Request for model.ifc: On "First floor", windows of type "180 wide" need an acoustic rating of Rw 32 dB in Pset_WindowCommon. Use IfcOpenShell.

First a look at what the model holds.

```python
import ifcopenshell
import ifcopenshell.util.element

model = ifcopenshell.open("model.ifc")
print(model.schema)
storey = next(s for s in model.by_type("IfcBuildingStorey") if s.Name == "First floor")
windows = [e for e in ifcopenshell.util.element.get_decomposition(storey) if e.is_a("IfcWindow")]
seen = {}
for e in windows:
    element_type = ifcopenshell.util.element.get_type(e)
    key = (element_type.Name if element_type != e and element_type else None, ifcopenshell.util.element.get_pset(e, "Pset_WindowCommon", "AcousticRating"))
    seen[key] = seen.get(key, 0) + 1
for (name, value), count in sorted(seen.items(), key=str):
    print(count, "x", name, "|", value)
```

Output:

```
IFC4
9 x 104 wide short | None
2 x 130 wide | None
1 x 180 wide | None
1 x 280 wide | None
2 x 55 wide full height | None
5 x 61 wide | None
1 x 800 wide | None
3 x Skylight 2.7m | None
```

```python
import ifcopenshell
import ifcopenshell.api.pset
import ifcopenshell.util.element

model = ifcopenshell.open("model.ifc")

storey = next(s for s in model.by_type("IfcBuildingStorey") if s.Name == "First floor")
windows = [e for e in ifcopenshell.util.element.get_decomposition(storey) if e.is_a("IfcWindow")]

count = 0
for e in windows:
    element_type = ifcopenshell.util.element.get_type(e)
    if element_type in (None, e) or element_type.Name != "180 wide":
        continue
    # add_pset returns the element's existing set when there is one.
    pset = ifcopenshell.api.pset.add_pset(model, product=e, name="Pset_WindowCommon")
    ifcopenshell.api.pset.edit_pset(model, pset=pset, properties={"AcousticRating": "Rw 32 dB"})
    count += 1

print(count, "windows updated")

model.write("model_rev.ifc")
```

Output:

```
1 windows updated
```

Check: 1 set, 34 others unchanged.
